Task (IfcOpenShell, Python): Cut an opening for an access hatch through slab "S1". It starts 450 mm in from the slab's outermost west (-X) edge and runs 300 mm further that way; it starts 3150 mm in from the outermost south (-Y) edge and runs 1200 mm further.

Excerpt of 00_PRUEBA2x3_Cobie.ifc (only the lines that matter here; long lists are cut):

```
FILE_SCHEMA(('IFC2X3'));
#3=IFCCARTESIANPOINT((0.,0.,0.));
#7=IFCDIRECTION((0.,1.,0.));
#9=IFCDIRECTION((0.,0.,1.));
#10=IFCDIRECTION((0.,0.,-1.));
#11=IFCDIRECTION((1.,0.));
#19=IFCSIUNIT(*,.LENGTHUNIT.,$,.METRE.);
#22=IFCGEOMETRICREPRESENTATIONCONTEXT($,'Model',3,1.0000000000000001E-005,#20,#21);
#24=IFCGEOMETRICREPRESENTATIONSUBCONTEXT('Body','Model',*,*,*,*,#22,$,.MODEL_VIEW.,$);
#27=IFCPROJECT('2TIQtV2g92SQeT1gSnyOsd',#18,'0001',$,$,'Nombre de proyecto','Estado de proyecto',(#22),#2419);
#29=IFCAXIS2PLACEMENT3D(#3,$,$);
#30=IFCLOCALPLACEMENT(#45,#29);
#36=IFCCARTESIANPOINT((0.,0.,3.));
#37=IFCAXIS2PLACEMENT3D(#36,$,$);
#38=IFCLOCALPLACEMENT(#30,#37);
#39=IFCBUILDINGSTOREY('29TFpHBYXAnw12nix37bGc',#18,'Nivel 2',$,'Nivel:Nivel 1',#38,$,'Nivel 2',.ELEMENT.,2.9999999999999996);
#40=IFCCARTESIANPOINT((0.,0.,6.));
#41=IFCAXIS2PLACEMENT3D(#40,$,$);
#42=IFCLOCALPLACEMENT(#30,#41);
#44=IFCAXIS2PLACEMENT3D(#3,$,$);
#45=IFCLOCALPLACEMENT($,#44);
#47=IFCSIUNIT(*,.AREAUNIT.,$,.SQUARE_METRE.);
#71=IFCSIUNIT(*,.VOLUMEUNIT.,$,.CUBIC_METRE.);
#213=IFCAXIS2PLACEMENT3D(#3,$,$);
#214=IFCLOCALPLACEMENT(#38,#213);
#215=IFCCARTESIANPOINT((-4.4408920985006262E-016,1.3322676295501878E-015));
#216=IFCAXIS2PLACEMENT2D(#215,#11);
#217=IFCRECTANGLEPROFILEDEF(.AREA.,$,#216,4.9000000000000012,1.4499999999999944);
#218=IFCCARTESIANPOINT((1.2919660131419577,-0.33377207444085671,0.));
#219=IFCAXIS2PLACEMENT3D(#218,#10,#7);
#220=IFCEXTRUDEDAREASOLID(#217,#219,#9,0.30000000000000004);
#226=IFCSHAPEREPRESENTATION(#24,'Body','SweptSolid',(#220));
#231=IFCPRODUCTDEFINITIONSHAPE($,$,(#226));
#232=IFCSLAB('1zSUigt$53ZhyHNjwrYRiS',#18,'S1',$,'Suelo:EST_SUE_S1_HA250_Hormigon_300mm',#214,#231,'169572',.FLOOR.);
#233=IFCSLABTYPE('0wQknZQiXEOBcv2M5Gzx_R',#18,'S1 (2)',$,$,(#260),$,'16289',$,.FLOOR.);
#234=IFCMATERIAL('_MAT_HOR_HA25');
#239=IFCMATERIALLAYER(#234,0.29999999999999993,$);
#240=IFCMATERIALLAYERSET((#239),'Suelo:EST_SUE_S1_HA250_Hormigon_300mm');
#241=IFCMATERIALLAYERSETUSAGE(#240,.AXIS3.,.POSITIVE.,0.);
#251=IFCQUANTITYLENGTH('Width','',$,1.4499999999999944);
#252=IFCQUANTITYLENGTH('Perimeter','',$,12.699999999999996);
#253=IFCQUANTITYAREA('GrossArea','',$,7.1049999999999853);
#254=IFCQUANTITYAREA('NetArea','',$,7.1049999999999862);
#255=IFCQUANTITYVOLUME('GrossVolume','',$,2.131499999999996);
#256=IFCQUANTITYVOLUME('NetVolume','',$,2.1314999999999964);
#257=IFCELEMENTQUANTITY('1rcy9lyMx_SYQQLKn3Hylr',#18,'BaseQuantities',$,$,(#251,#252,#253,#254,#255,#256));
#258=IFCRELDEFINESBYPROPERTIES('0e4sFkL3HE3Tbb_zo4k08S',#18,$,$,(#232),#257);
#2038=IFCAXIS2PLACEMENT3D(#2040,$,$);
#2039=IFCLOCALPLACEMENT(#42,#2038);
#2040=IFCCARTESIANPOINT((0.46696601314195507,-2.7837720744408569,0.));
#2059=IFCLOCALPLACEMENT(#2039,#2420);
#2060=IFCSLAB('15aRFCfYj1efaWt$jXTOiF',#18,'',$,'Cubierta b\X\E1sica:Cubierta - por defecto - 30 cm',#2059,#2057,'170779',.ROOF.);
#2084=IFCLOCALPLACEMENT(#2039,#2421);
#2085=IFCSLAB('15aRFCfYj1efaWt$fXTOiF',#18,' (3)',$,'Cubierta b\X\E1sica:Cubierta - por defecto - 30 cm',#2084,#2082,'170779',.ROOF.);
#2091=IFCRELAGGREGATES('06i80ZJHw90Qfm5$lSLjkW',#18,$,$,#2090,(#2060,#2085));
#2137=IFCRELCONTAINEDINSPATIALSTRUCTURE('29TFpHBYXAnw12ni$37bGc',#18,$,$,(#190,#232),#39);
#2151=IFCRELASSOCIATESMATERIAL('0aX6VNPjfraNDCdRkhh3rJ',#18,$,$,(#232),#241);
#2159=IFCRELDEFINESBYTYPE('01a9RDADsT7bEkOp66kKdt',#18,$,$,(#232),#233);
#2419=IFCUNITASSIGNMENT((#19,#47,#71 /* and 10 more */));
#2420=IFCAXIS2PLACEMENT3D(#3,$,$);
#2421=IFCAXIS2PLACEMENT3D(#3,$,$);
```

```python
import numpy as np
import ifcopenshell
import ifcopenshell.api.feature
import ifcopenshell.api.geometry
import ifcopenshell.api.pset
import ifcopenshell.api.root
import ifcopenshell.geom
import ifcopenshell.util.element
import ifcopenshell.util.placement
import ifcopenshell.util.representation
import ifcopenshell.util.shape
import ifcopenshell.util.unit

model = ifcopenshell.open("00_PRUEBA2x3_Cobie.ifc")
unit_scale = ifcopenshell.util.unit.calculate_unit_scale(model)
area_scale = ifcopenshell.util.unit.calculate_unit_scale(model, "AREAUNIT")
volume_scale = ifcopenshell.util.unit.calculate_unit_scale(model, "VOLUMEUNIT")
settings = ifcopenshell.geom.settings()


def volume(element):
    """Net volume in cubic metres, openings subtracted."""
    shape = ifcopenshell.geom.create_shape(settings, element)
    return ifcopenshell.util.shape.get_volume(shape.geometry)


slab = model.by_guid("1zSUigt$53ZhyHNjwrYRiS")
before = volume(slab)

# Extent in the slab's own axes, in metres. The edges named are its -X and -Y sides.
slab_shape = ifcopenshell.geom.create_shape(settings, slab)
vertices = ifcopenshell.util.shape.get_vertices(slab_shape.geometry)
x_min, y_min, bottom = vertices.min(axis=0)
top = vertices[:, 2].max()

opening = ifcopenshell.api.root.create_entity(model, ifc_class="IfcOpeningElement", name="Access hatch opening")
context = ifcopenshell.util.representation.get_context(model, "Model", "Body", "MODEL_VIEW")
width, depth = 0.3, 1.2
outline = [(0.0, 0.0), (width, 0.0), (width, depth), (0.0, depth), (0.0, 0.0)]
# Overshoot both faces by 50 mm so the cut is clean.
shape = ifcopenshell.api.geometry.add_slab_representation(
    model, context=context, depth=top - bottom + 0.1, polyline=outline
)
ifcopenshell.api.geometry.assign_representation(model, product=opening, representation=shape)

matrix = ifcopenshell.util.placement.get_local_placement(slab.ObjectPlacement)
matrix[:, 3] = matrix @ np.append(np.array([x_min + 0.45, y_min + 3.15, bottom - 0.05]) / unit_scale, 1.0)
ifcopenshell.api.geometry.edit_object_placement(model, product=opening, matrix=matrix, is_si=False)
ifcopenshell.api.feature.add_feature(model, feature=opening, element=slab)

after = volume(slab)

# Update the slab's stored quantities.
qto = model.by_id(ifcopenshell.util.element.get_pset(slab, "BaseQuantities", should_inherit=False)["id"])
ifcopenshell.api.pset.edit_qto(model, qto=qto, properties={
    "NetArea": after / (top - bottom) / area_scale,
    "NetVolume": after / volume_scale,
})

print(f"slab volume {before:.3f} -> {after:.3f} m3")

model.write("00_PRUEBA2x3_Cobie_v2.ifc")
```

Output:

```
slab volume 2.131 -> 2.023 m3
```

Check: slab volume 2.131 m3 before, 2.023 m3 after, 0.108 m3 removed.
